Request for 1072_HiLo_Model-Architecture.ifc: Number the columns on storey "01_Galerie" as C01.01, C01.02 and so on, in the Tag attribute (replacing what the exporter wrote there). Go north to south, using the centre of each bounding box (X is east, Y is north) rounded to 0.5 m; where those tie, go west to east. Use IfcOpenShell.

First a look at what the model holds.

```python
import ifcopenshell
import ifcopenshell.util.element
import ifcopenshell.util.placement

model = ifcopenshell.open("1072_HiLo_Model-Architecture.ifc")
print(model.schema)
storey = next(s for s in model.by_type("IfcBuildingStorey") if s.Name == "01_Galerie")
columns = [e for e in ifcopenshell.util.element.get_decomposition(storey) if e.is_a("IfcColumn")]
for e in sorted(columns, key=lambda e: e.id()):
    origin = ifcopenshell.util.placement.get_local_placement(e.ObjectPlacement)[:3, 3]
    print(e.id(), e.Tag, e.Name, origin.round(2) + 0.0, sep=" | ")
```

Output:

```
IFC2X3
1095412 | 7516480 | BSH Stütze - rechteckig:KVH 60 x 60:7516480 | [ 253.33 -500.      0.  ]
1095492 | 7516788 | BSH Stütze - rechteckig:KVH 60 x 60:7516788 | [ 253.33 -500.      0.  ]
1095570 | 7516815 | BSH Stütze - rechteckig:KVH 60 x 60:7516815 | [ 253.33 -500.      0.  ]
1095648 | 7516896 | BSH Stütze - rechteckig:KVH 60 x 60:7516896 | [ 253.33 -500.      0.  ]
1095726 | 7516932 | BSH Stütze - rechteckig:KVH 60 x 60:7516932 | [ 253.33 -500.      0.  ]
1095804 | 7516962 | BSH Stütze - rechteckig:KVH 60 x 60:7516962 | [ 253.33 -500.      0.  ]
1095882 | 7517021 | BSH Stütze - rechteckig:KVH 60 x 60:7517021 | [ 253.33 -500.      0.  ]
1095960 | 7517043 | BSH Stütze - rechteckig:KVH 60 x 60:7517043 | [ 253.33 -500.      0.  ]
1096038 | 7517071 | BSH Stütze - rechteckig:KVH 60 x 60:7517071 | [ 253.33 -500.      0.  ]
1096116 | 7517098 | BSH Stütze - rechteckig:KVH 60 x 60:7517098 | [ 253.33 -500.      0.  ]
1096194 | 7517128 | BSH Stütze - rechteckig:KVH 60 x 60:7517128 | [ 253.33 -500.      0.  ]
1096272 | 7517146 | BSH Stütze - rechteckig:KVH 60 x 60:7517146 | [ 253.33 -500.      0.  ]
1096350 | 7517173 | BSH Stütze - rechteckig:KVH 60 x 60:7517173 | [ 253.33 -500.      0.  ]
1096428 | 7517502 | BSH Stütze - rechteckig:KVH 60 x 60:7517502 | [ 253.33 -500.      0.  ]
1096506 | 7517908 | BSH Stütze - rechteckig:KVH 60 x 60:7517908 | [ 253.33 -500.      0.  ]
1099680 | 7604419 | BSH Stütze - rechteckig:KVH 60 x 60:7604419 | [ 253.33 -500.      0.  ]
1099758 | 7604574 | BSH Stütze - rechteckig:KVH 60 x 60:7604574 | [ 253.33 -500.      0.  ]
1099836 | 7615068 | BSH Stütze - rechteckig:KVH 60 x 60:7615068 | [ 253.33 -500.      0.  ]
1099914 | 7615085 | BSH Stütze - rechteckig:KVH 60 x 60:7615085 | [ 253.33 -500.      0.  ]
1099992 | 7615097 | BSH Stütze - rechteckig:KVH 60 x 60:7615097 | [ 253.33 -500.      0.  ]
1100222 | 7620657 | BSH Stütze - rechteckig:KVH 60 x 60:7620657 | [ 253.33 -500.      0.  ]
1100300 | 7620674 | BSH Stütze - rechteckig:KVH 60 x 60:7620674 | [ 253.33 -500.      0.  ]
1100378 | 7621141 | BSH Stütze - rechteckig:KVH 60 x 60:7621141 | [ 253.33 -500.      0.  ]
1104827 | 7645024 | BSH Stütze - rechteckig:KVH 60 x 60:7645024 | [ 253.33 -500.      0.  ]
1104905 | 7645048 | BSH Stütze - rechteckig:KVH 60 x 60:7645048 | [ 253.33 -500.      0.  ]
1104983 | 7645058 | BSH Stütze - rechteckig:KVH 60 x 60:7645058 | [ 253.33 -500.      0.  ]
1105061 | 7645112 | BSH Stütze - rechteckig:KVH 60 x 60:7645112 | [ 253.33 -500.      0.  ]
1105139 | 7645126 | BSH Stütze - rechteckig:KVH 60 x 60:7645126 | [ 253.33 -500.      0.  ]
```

```python
import ifcopenshell
import ifcopenshell.geom
import ifcopenshell.util.element
import ifcopenshell.util.shape

model = ifcopenshell.open("1072_HiLo_Model-Architecture.ifc")
settings = ifcopenshell.geom.settings()
settings.set("use-world-coords", True)


def centre(element):
    shape = ifcopenshell.geom.create_shape(settings, element)
    return ifcopenshell.util.shape.get_bbox_centroid(shape.geometry)


storey = next(s for s in model.by_type("IfcBuildingStorey") if s.Name == "01_Galerie")
columns = [e for e in ifcopenshell.util.element.get_decomposition(storey) if e.is_a("IfcColumn")]

# Insertion points can sit at a corner or the storey origin, so sort by the geometry (in metres).
centres = {e: centre(e) for e in columns}
columns.sort(key=lambda e: (-round(centres[e][1] / 0.5), centres[e][0]))

for i, e in enumerate(columns, start=1):
    number = f"C01.{i:02d}"
    e.Tag = number
    print(e.id(), number)

model.write("1072_HiLo_Model-Architecture_updated.ifc")
```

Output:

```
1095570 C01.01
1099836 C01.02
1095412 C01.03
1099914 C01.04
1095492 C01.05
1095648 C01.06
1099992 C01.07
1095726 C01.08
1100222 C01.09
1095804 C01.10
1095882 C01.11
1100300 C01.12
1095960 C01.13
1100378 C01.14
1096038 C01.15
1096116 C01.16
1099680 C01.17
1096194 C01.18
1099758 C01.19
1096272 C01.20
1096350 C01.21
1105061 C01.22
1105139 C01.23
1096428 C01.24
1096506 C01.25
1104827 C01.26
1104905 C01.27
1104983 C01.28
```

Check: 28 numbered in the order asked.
